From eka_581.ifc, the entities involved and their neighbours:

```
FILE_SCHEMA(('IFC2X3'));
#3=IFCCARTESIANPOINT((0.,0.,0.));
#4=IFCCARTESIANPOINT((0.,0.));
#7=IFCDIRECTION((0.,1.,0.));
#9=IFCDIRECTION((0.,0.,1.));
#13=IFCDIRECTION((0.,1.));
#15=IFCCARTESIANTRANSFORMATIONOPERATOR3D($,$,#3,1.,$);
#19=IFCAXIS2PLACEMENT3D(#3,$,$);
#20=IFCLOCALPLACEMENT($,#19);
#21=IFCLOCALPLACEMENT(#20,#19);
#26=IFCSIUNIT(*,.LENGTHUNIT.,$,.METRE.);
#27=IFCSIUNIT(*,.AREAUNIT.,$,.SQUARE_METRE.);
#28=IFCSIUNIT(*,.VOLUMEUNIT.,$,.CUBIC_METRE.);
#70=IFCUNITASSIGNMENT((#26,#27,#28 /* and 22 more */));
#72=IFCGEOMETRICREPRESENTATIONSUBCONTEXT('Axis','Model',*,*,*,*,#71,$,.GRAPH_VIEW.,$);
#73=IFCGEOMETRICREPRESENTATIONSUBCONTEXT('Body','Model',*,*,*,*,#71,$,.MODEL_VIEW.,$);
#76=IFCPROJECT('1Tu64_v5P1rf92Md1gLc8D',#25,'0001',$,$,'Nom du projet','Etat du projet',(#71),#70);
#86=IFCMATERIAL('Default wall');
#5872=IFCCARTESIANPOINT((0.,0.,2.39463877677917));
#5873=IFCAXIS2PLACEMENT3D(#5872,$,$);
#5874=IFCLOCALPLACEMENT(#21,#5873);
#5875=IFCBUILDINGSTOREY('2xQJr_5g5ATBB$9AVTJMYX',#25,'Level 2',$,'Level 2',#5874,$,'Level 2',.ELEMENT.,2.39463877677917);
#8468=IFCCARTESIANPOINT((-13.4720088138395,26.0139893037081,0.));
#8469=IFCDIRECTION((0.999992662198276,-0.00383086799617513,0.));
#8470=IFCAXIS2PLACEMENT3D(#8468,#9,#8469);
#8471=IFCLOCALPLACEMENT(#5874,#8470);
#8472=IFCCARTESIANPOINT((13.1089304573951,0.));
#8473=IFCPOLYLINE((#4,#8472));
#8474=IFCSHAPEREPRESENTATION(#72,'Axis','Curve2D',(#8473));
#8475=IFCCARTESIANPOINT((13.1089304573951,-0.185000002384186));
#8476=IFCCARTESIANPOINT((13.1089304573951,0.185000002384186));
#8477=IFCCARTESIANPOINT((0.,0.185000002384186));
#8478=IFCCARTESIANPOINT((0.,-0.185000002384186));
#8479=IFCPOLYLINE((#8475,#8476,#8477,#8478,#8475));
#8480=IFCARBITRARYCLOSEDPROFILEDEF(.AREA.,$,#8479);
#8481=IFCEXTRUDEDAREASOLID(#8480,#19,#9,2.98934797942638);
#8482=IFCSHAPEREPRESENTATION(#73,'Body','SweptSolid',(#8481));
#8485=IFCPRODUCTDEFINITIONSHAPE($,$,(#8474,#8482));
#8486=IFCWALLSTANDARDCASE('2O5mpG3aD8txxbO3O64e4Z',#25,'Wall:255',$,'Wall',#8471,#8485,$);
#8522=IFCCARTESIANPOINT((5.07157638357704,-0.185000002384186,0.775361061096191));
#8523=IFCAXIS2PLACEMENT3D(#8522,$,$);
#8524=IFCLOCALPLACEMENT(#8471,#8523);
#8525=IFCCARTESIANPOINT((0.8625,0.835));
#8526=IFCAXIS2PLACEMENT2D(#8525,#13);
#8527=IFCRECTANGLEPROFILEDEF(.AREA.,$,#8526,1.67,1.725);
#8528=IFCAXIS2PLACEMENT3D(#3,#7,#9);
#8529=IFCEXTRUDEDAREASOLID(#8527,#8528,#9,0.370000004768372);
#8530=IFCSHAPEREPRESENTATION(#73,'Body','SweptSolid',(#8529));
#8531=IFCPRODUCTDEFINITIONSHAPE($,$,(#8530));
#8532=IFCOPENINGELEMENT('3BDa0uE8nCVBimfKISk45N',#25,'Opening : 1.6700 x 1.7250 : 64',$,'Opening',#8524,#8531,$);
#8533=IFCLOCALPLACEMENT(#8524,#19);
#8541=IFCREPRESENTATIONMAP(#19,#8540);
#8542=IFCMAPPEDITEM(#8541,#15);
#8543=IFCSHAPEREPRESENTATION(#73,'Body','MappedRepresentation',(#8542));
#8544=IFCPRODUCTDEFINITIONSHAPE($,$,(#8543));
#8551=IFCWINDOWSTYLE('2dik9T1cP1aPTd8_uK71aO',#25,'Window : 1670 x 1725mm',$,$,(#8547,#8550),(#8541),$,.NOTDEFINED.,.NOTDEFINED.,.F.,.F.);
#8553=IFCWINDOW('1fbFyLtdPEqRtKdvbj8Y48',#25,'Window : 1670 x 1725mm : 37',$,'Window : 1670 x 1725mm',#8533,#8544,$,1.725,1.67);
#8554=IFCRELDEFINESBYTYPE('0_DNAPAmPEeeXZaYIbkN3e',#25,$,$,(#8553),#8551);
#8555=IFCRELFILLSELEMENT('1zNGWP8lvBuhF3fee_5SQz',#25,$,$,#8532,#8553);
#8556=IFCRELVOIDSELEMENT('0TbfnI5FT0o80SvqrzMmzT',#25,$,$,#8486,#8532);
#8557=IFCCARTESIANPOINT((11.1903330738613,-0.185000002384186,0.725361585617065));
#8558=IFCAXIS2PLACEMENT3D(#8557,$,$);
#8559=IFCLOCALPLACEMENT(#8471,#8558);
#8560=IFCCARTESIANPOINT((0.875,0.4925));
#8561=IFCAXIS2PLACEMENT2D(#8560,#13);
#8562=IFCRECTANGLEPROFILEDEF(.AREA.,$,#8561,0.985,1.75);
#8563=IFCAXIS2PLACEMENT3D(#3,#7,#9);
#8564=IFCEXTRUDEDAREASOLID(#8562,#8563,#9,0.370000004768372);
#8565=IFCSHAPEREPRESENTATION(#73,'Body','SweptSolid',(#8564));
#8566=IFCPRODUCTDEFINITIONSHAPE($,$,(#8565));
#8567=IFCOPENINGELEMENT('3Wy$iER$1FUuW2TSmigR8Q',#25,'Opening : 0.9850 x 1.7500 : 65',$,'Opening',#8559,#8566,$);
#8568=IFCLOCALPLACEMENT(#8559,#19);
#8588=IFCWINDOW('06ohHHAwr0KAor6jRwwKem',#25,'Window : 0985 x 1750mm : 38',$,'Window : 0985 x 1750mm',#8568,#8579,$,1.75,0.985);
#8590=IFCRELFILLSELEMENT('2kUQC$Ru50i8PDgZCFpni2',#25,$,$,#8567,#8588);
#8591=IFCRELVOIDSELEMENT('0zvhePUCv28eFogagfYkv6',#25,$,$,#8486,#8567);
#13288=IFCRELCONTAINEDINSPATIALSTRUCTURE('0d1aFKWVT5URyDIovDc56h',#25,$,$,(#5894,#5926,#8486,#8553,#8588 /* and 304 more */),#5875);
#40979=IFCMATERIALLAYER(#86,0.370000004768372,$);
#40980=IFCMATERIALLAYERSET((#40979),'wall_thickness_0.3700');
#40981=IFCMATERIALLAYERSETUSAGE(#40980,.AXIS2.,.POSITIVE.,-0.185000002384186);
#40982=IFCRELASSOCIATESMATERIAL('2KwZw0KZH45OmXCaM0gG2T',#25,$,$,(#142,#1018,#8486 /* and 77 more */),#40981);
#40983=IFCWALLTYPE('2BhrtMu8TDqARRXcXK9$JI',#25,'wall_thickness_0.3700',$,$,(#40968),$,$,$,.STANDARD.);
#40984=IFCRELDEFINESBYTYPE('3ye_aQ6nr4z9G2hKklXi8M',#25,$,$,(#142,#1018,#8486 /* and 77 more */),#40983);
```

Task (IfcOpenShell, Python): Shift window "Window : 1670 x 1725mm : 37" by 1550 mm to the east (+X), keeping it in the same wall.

```python
import ifcopenshell
import ifcopenshell.api.geometry
import ifcopenshell.util.placement

model = ifcopenshell.open("eka_581.ifc")

window = model.by_guid("1fbFyLtdPEqRtKdvbj8Y48")
opening = window.FillsVoids[0].RelatingOpeningElement
wall = opening.VoidsElements[0].RelatingBuildingElement

wall_matrix = ifcopenshell.util.placement.get_local_placement(wall.ObjectPlacement)
shift = wall_matrix[:3, 0] * 1.55
before = ifcopenshell.util.placement.get_local_placement(window.ObjectPlacement)[:3, 3].copy()

# The window is placed relative to its opening, so it follows when the opening moves.
matrix = ifcopenshell.util.placement.get_local_placement(opening.ObjectPlacement)
matrix[:3, 3] += shift
ifcopenshell.api.geometry.edit_object_placement(
    model, product=opening, matrix=matrix, is_si=False, should_transform_children=True
)

after = ifcopenshell.util.placement.get_local_placement(window.ObjectPlacement)[:3, 3]
print("window moved by", (after - before).round(3) + 0.0)

model.write("eka_581_updated.ifc")
```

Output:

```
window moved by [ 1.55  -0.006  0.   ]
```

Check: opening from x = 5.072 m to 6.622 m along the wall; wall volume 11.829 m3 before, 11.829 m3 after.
